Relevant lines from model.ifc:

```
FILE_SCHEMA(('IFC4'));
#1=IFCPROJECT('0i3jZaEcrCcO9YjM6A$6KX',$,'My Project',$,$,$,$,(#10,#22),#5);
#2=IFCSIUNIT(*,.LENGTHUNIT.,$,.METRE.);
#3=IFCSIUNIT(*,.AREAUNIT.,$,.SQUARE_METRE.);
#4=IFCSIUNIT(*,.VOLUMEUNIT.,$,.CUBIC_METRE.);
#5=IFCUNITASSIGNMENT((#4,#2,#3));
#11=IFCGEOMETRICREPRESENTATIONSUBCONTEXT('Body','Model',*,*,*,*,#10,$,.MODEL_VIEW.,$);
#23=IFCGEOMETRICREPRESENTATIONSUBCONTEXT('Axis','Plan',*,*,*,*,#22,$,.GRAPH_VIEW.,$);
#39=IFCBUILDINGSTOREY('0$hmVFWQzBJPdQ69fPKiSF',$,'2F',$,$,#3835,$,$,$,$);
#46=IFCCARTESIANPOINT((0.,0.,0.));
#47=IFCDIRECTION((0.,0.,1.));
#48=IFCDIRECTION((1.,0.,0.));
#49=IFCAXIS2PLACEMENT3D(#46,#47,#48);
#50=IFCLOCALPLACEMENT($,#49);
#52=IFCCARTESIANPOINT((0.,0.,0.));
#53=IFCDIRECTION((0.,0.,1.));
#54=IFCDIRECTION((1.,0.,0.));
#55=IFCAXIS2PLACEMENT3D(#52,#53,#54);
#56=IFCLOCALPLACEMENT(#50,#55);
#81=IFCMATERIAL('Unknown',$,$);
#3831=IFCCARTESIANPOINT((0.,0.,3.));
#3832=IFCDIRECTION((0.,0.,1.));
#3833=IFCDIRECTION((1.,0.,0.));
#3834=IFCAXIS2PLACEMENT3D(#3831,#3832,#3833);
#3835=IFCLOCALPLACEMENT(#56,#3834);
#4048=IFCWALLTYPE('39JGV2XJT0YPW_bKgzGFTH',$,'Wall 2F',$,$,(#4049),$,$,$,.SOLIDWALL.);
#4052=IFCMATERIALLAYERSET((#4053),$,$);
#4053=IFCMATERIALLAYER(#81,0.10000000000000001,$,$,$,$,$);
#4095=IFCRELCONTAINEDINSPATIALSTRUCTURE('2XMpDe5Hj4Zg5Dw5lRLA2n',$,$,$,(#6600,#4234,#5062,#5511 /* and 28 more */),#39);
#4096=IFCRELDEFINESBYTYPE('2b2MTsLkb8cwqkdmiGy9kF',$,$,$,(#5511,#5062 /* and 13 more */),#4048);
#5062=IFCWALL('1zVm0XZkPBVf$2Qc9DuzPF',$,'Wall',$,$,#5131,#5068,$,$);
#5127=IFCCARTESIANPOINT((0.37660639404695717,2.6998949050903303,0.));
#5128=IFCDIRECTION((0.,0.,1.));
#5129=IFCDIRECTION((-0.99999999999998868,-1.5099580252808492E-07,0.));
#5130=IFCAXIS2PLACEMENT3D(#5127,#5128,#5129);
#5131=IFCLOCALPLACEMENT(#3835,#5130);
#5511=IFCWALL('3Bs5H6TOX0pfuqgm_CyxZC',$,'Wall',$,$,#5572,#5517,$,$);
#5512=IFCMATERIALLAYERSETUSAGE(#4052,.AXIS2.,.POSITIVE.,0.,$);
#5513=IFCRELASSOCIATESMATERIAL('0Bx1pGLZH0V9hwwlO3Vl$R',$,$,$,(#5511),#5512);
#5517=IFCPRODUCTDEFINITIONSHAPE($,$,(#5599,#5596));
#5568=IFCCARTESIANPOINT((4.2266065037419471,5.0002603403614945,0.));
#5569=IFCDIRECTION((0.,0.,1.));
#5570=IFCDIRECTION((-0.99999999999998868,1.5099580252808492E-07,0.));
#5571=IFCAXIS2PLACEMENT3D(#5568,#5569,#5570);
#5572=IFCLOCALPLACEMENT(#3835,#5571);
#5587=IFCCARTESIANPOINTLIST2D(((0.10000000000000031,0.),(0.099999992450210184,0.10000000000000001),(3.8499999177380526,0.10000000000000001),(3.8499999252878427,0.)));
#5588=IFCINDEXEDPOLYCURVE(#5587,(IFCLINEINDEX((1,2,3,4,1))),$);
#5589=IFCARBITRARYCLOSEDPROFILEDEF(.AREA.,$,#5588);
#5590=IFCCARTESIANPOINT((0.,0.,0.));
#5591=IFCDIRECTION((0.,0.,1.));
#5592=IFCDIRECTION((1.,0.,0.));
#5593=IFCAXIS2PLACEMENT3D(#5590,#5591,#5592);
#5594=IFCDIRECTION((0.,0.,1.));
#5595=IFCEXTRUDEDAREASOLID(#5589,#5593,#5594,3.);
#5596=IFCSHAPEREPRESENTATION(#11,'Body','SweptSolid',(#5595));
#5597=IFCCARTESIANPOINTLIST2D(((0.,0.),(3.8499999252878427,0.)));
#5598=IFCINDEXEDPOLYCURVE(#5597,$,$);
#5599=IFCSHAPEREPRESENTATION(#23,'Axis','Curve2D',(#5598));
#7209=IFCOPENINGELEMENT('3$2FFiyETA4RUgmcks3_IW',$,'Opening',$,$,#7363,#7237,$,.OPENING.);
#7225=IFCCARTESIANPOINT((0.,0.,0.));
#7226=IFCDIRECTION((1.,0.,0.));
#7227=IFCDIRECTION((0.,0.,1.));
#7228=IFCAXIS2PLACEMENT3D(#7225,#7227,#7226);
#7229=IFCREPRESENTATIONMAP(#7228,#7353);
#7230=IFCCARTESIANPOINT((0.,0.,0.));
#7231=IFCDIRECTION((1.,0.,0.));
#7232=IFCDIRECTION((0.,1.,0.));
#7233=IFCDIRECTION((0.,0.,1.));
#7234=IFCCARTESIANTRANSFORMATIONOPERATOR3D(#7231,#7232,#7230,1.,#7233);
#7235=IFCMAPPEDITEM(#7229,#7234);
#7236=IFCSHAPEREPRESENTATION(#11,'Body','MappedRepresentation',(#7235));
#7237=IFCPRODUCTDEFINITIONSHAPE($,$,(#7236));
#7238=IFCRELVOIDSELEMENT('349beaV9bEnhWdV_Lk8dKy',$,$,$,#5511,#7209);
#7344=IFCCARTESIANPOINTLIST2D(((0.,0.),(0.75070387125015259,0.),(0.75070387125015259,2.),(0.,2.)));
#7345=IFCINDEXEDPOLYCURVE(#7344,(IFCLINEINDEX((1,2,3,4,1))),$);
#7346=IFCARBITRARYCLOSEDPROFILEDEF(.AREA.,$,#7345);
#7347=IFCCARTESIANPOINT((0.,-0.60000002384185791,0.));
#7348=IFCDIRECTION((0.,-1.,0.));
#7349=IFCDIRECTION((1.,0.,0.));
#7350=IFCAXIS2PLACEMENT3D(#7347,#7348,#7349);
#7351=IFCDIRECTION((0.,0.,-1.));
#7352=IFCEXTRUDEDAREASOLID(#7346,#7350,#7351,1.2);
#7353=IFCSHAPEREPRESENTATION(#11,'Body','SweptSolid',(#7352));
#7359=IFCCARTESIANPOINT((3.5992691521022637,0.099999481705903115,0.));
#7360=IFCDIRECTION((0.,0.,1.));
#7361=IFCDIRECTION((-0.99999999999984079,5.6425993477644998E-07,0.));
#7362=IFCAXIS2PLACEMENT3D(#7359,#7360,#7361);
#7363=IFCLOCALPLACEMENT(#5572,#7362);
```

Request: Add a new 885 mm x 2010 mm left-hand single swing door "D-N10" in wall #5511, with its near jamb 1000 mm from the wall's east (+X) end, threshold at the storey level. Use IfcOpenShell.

```python
import numpy as np
import ifcopenshell
import ifcopenshell.api.feature
import ifcopenshell.api.geometry
import ifcopenshell.api.root
import ifcopenshell.api.spatial
import ifcopenshell.geom
import ifcopenshell.util.element
import ifcopenshell.util.placement
import ifcopenshell.util.representation
import ifcopenshell.util.shape
import ifcopenshell.util.unit

model = ifcopenshell.open("model.ifc")
unit_scale = ifcopenshell.util.unit.calculate_unit_scale(model)
settings = ifcopenshell.geom.settings()


def volume(element):
    """Net volume in cubic metres, openings subtracted."""
    shape = ifcopenshell.geom.create_shape(settings, element)
    return ifcopenshell.util.shape.get_volume(shape.geometry)


wall = model.by_id(5511)
storey = ifcopenshell.util.element.get_container(wall, ifc_class="IfcBuildingStorey")
context = ifcopenshell.util.representation.get_context(model, "Model", "Body", "MODEL_VIEW")
before = volume(wall)

width, height, from_end, sill = 0.885, 2.01, 1, 0.0  # metres

# The wall runs along its own X axis, and the end named is its -X end.
wall_shape = ifcopenshell.geom.create_shape(settings, wall)
x, y, z = ifcopenshell.util.shape.get_vertices(wall_shape.geometry).T
start = x.min() + from_end
face, thickness = float(y.min()), float(y.max() - y.min())
wall_matrix = ifcopenshell.util.placement.get_local_placement(wall.ObjectPlacement)
level = ifcopenshell.util.placement.get_local_placement(storey.ObjectPlacement)[2, 3]


def in_wall(x, y):
    """Placement at x, y metres in the wall's axes, at sill height."""
    matrix = wall_matrix.copy()
    matrix[:, 3] = wall_matrix @ np.array([x / unit_scale, y / unit_scale, 0.0, 1.0])
    matrix[2, 3] = level + sill / unit_scale
    return matrix


# Opening: a box that overshoots both wall faces by 50 mm.
opening = ifcopenshell.api.root.create_entity(model, ifc_class="IfcOpeningElement", predefined_type="OPENING")
box = ifcopenshell.api.geometry.add_wall_representation(
    model, context=context, length=width, height=height, thickness=thickness + 0.1
)
ifcopenshell.api.geometry.assign_representation(model, product=opening, representation=box)
ifcopenshell.api.geometry.edit_object_placement(model, product=opening, matrix=in_wall(start, face - 0.05), is_si=False)
ifcopenshell.api.feature.add_feature(model, feature=opening, element=wall)

door = ifcopenshell.api.root.create_entity(model, ifc_class="IfcDoor", name="D-N10", predefined_type="DOOR")
door.OverallWidth, door.OverallHeight = width / unit_scale, height / unit_scale
door.OperationType = "SINGLE_SWING_LEFT"
body = ifcopenshell.api.geometry.add_door_representation(
    model,
    context=context,
    overall_width=door.OverallWidth,
    overall_height=door.OverallHeight,
    operation_type="SINGLE_SWING_LEFT",
    lining_properties={"LiningDepth": thickness / unit_scale, "ThresholdDepth": thickness / unit_scale},
)
ifcopenshell.api.geometry.assign_representation(model, product=door, representation=body)
ifcopenshell.api.spatial.assign_container(model, products=[door], relating_structure=storey)
ifcopenshell.api.feature.add_filling(model, opening=opening, element=door)

# The lining spans the wall, so the door starts at the wall face.
ifcopenshell.api.geometry.edit_object_placement(model, product=door, matrix=in_wall(start, face), is_si=False)

after = volume(wall)

print(f"wall volume {before:.3f} -> {after:.3f} m3")

model.write("model_updated.ifc")
```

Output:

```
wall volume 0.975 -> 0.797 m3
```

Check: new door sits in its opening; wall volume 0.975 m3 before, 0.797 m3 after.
